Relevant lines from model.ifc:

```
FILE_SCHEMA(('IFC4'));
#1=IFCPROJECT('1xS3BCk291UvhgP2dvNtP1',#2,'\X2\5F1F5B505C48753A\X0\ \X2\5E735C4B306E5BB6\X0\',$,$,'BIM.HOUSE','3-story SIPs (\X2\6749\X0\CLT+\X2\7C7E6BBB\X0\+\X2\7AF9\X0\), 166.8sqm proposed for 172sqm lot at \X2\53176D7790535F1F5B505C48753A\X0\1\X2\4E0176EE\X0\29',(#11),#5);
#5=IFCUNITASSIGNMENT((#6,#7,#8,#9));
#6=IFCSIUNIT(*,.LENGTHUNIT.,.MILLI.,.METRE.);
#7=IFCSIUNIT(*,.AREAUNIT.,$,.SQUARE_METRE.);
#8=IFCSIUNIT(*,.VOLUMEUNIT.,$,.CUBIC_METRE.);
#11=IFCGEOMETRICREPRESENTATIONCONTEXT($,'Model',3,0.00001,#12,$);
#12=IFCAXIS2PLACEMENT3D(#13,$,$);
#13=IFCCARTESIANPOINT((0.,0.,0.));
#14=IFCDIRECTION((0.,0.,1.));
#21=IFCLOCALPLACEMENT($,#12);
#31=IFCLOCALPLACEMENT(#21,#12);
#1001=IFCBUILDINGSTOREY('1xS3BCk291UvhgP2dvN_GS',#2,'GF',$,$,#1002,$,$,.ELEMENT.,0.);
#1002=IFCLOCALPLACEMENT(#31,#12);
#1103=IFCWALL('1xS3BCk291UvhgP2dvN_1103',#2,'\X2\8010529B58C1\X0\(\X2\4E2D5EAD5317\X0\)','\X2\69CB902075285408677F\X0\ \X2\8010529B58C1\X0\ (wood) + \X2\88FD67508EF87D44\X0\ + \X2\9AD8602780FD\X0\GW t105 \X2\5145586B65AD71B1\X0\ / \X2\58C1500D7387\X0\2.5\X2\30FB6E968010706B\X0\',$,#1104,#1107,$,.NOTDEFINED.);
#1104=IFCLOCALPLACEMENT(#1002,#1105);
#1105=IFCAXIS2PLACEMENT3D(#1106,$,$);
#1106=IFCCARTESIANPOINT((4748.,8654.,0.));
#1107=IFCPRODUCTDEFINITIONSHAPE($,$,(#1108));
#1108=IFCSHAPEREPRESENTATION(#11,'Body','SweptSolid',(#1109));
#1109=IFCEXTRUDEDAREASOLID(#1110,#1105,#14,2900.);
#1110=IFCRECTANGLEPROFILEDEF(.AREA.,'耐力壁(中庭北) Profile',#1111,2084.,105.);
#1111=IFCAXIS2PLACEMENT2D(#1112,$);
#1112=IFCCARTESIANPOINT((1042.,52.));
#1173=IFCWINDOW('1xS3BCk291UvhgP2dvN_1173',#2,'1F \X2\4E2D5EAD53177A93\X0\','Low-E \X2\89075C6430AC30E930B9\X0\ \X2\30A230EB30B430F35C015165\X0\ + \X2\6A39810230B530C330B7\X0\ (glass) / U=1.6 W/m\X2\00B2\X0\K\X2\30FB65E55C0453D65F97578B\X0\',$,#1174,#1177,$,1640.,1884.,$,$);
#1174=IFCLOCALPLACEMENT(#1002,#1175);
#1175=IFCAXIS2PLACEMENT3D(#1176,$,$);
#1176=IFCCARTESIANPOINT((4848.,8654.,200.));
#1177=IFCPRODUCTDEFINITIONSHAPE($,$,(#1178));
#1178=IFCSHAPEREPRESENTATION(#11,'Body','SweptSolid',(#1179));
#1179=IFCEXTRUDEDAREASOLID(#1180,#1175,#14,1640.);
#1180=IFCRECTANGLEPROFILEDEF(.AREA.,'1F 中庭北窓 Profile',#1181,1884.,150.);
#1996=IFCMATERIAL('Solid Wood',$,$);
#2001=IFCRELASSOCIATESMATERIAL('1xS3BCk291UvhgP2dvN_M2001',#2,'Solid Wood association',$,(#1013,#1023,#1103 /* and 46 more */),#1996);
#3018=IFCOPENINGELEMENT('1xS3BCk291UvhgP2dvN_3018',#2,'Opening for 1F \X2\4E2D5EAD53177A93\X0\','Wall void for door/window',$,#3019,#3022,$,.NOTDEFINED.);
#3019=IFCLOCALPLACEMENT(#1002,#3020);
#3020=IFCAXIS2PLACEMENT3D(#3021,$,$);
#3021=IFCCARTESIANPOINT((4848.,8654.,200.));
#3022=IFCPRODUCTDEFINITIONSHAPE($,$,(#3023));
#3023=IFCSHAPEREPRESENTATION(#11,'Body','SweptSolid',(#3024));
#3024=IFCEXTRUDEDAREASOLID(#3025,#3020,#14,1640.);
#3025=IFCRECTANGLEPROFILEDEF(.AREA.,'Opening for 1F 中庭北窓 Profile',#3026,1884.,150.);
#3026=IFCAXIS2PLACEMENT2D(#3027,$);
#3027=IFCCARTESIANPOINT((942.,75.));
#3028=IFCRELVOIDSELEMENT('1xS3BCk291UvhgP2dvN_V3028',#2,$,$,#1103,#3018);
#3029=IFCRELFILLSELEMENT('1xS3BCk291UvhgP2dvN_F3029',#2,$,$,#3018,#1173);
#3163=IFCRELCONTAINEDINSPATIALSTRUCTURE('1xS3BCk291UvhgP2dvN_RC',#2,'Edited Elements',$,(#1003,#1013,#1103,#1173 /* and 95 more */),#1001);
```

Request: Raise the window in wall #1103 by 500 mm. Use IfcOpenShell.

```python
import numpy as np
import ifcopenshell
import ifcopenshell.api.geometry
import ifcopenshell.util.placement
import ifcopenshell.util.unit

model = ifcopenshell.open("model.ifc")
unit_scale = ifcopenshell.util.unit.calculate_unit_scale(model)

window = model.by_id(1173)
opening = window.FillsVoids[0].RelatingOpeningElement
dz = 0.5 / unit_scale

shift = np.array([0.0, 0.0, dz])
# The window is not placed relative to its opening, so move both.
for product in (opening, window):
    matrix = ifcopenshell.util.placement.get_local_placement(product.ObjectPlacement)
    matrix[:3, 3] += shift
    ifcopenshell.api.geometry.edit_object_placement(model, product=product, matrix=matrix, is_si=False)

print(f"moved by {dz * unit_scale:+.3f} m")

model.write("model_v2.ifc")
```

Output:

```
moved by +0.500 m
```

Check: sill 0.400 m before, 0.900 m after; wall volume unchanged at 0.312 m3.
